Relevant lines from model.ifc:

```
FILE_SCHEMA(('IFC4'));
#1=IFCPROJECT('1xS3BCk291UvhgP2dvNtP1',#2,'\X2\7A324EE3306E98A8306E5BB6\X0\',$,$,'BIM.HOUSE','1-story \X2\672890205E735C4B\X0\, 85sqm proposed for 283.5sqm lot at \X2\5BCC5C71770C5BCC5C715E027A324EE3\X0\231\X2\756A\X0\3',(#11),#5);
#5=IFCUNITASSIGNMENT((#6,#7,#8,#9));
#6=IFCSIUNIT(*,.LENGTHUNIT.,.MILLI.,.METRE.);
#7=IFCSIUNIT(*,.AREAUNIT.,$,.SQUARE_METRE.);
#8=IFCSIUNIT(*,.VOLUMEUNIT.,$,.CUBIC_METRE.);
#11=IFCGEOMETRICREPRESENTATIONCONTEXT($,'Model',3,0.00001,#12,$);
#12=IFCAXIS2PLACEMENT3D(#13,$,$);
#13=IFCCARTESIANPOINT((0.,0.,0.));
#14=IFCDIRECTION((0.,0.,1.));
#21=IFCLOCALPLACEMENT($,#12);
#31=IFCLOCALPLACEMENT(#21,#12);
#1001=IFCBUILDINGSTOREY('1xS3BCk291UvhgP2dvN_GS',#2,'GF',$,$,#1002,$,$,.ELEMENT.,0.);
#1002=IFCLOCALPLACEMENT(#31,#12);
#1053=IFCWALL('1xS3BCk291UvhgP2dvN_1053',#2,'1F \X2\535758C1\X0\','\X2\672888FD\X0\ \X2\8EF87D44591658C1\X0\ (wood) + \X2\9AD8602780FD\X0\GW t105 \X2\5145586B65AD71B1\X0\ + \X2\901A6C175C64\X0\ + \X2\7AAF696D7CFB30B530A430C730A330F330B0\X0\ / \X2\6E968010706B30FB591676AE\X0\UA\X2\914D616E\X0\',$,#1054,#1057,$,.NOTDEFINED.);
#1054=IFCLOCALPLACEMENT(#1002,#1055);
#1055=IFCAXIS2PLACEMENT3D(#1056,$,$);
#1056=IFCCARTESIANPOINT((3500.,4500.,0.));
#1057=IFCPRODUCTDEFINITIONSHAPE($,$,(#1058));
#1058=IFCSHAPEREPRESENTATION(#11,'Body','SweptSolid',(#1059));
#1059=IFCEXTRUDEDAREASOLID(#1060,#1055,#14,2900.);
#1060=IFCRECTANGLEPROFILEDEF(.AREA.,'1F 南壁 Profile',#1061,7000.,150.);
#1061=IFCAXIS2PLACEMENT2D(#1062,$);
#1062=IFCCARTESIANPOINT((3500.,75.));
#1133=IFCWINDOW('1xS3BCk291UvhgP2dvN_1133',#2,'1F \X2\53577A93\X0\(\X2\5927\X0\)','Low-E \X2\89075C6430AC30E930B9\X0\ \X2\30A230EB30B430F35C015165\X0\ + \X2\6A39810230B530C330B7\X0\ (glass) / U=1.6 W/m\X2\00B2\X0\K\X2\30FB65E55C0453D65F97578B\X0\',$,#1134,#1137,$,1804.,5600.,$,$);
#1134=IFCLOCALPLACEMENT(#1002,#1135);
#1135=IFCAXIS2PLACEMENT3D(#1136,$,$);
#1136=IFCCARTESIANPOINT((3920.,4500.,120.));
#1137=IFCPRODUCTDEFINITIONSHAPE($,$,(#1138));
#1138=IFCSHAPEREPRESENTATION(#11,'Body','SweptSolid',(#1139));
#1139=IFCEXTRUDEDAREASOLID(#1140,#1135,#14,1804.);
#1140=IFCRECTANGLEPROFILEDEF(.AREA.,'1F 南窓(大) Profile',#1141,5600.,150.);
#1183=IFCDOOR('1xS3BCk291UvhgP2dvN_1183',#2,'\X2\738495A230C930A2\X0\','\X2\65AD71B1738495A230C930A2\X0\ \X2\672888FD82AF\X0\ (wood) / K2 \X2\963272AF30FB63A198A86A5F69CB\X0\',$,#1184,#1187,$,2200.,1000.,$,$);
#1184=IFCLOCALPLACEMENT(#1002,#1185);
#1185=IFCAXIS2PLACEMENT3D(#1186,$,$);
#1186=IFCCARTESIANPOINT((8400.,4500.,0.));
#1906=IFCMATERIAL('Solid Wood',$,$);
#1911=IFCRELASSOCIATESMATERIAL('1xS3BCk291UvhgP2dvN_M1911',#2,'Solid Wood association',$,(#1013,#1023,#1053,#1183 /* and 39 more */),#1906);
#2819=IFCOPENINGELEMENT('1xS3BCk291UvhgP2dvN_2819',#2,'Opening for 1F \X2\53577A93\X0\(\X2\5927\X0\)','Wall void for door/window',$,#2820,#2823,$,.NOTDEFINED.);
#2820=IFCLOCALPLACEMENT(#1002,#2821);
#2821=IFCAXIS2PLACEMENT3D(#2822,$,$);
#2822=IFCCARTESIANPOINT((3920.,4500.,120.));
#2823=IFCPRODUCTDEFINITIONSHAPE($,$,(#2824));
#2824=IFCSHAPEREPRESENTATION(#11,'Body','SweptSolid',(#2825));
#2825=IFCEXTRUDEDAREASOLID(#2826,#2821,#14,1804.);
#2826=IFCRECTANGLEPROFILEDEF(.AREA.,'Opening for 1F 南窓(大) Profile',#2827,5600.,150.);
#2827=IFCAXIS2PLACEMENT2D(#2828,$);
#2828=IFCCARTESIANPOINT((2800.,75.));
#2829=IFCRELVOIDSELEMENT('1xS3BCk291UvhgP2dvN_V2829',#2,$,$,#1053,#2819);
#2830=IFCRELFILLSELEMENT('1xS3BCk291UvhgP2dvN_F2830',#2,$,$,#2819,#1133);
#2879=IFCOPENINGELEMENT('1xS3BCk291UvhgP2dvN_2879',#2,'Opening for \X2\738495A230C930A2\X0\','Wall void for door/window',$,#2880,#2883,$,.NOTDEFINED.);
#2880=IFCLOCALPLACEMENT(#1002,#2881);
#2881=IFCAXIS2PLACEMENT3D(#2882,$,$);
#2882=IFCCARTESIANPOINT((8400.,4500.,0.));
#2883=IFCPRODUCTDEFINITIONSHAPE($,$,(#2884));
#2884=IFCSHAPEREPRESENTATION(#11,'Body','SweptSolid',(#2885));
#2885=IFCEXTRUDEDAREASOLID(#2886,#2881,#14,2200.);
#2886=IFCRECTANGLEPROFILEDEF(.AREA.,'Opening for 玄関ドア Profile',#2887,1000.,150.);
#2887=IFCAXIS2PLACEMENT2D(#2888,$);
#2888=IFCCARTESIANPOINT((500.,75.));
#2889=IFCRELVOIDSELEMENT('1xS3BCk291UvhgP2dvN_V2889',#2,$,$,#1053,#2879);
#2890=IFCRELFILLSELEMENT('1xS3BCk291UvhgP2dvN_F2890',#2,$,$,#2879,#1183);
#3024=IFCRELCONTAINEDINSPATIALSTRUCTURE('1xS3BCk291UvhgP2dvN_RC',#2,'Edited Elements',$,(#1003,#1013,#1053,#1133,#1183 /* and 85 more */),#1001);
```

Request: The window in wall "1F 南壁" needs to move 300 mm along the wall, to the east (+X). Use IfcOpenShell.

```python
import ifcopenshell
import ifcopenshell.api.geometry
import ifcopenshell.util.placement
import ifcopenshell.util.unit

model = ifcopenshell.open("model.ifc")
unit_scale = ifcopenshell.util.unit.calculate_unit_scale(model)

window = model.by_guid("1xS3BCk291UvhgP2dvN_1133")
opening = window.FillsVoids[0].RelatingOpeningElement
wall = opening.VoidsElements[0].RelatingBuildingElement

wall_matrix = ifcopenshell.util.placement.get_local_placement(wall.ObjectPlacement)
shift = wall_matrix[:3, 0] * 0.3 / unit_scale
before = ifcopenshell.util.placement.get_local_placement(window.ObjectPlacement)[:3, 3].copy()

# The window is not placed relative to its opening, so move both.
for product in (opening, window):
    matrix = ifcopenshell.util.placement.get_local_placement(product.ObjectPlacement)
    matrix[:3, 3] += shift
    ifcopenshell.api.geometry.edit_object_placement(model, product=product, matrix=matrix, is_si=False)

after = ifcopenshell.util.placement.get_local_placement(window.ObjectPlacement)[:3, 3]
print("window moved by", (after - before).round(3) + 0.0)

model.write("model_v2.ifc")
```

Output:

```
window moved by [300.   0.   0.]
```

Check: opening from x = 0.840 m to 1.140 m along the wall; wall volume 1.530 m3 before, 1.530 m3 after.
